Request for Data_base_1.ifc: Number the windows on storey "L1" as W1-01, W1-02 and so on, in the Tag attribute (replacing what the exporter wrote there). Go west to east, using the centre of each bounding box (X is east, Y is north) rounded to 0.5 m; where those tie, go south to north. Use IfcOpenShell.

First a look at what the model holds.

```python
import ifcopenshell
import ifcopenshell.util.element
import ifcopenshell.util.placement

model = ifcopenshell.open("Data_base_1.ifc")
print(model.schema)
storey = next(s for s in model.by_type("IfcBuildingStorey") if s.Name == "L1")
windows = [e for e in ifcopenshell.util.element.get_decomposition(storey) if e.is_a("IfcWindow")]
for e in sorted(windows, key=lambda e: e.id()):
    origin = ifcopenshell.util.placement.get_local_placement(e.ObjectPlacement)[:3, 3]
    print(e.id(), e.Tag, e.Name, origin.round(2) + 0.0, sep=" | ")
```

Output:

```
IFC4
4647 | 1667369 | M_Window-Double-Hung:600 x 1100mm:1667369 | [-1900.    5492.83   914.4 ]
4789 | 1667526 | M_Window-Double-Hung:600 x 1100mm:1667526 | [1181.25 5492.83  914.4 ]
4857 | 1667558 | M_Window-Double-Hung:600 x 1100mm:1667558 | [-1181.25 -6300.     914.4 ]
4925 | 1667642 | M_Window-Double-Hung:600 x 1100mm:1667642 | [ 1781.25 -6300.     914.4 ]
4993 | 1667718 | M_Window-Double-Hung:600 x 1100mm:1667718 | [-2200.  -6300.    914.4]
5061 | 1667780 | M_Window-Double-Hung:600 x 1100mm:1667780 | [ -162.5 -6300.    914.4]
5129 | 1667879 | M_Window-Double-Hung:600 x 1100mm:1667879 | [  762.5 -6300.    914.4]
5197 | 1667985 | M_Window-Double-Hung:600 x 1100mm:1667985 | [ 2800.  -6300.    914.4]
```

```python
import ifcopenshell
import ifcopenshell.geom
import ifcopenshell.util.element
import ifcopenshell.util.shape

model = ifcopenshell.open("Data_base_1.ifc")
settings = ifcopenshell.geom.settings()
settings.set("use-world-coords", True)


def centre(element):
    shape = ifcopenshell.geom.create_shape(settings, element)
    return ifcopenshell.util.shape.get_bbox_centroid(shape.geometry)


storey = next(s for s in model.by_type("IfcBuildingStorey") if s.Name == "L1")
windows = [e for e in ifcopenshell.util.element.get_decomposition(storey) if e.is_a("IfcWindow")]

# Insertion points can sit at a corner or the storey origin, so sort by the geometry (in metres).
centres = {e: centre(e) for e in windows}
windows.sort(key=lambda e: (round(centres[e][0] / 0.5), centres[e][1]))

for i, e in enumerate(windows, start=1):
    number = f"W1-{i:02d}"
    e.Tag = number
    print(e.id(), number)

model.write("Data_base_1_edited.ifc")
```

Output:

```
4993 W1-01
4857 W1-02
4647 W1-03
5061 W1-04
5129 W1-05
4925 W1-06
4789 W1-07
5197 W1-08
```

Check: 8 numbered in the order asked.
